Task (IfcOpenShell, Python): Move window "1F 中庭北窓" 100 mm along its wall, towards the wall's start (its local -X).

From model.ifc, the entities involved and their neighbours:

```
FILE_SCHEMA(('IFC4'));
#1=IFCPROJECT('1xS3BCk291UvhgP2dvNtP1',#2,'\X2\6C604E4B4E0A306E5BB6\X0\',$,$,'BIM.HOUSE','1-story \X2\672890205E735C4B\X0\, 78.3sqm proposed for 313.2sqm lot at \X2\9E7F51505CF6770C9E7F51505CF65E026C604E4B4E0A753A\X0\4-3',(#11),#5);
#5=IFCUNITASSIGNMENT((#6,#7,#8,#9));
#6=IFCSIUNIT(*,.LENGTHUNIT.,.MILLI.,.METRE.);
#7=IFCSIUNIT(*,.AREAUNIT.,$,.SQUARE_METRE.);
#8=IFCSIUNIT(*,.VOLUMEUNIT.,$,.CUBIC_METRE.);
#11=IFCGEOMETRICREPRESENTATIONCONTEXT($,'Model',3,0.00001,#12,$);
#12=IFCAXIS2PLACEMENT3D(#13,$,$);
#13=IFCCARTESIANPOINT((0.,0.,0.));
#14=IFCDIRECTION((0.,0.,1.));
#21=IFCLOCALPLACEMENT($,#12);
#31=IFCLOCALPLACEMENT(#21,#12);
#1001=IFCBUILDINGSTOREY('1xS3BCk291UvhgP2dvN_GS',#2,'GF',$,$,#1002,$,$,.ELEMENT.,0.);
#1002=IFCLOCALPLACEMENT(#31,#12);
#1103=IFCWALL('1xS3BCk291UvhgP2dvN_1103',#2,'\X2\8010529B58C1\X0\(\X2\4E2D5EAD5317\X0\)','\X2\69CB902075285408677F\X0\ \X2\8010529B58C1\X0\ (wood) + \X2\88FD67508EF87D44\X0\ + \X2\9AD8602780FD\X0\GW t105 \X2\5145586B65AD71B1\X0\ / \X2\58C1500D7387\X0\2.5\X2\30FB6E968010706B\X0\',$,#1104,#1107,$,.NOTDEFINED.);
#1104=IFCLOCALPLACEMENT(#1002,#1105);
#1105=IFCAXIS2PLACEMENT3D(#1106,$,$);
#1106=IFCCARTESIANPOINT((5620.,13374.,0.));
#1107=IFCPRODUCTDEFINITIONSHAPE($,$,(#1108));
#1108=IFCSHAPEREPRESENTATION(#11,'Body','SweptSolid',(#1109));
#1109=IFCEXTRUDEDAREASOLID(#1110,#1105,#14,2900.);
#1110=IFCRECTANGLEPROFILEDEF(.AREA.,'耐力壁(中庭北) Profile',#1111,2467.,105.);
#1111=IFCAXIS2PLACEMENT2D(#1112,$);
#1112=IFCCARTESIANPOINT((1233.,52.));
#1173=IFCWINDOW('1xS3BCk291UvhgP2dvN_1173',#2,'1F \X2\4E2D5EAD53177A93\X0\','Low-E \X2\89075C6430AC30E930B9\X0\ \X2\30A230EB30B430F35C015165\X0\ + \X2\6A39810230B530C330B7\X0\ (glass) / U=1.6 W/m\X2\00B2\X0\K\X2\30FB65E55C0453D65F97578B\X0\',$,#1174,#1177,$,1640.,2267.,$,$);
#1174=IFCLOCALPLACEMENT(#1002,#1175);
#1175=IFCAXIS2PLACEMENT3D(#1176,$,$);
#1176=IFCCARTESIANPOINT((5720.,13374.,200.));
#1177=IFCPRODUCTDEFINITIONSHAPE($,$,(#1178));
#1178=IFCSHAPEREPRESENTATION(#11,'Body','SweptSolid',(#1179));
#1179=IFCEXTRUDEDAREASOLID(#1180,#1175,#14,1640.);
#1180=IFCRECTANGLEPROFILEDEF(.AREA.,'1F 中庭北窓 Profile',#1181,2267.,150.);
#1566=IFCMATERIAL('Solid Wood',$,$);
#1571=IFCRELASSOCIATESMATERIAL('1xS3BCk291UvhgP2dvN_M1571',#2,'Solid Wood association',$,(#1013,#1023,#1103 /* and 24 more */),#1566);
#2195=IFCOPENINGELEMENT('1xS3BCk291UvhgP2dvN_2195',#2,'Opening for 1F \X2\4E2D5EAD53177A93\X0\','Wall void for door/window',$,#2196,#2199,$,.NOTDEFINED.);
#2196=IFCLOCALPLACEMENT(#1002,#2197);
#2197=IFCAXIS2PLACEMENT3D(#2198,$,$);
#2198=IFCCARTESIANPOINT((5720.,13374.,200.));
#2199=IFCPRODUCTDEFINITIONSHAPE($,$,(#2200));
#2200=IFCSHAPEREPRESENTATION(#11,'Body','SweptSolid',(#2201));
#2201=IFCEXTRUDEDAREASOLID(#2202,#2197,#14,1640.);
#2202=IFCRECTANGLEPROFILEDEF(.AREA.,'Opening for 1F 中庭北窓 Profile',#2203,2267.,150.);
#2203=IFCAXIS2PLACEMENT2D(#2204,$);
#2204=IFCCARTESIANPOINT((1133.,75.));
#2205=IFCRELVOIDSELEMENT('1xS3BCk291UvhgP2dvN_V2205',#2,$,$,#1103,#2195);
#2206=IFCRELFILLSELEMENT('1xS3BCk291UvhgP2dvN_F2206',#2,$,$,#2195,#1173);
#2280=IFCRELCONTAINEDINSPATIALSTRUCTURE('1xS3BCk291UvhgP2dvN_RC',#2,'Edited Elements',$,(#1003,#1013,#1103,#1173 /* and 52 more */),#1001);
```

```python
import ifcopenshell
import ifcopenshell.api.geometry
import ifcopenshell.util.placement

model = ifcopenshell.open("model.ifc")

window = model.by_guid("1xS3BCk291UvhgP2dvN_1173")
opening = window.FillsVoids[0].RelatingOpeningElement
wall = opening.VoidsElements[0].RelatingBuildingElement

wall_matrix = ifcopenshell.util.placement.get_local_placement(wall.ObjectPlacement)
shift = wall_matrix[:3, 0] * -100.0
before = ifcopenshell.util.placement.get_local_placement(window.ObjectPlacement)[:3, 3].copy()

# The window is not placed relative to its opening, so move both.
for product in (opening, window):
    matrix = ifcopenshell.util.placement.get_local_placement(product.ObjectPlacement)
    matrix[:3, 3] += shift
    ifcopenshell.api.geometry.edit_object_placement(model, product=product, matrix=matrix, is_si=False)

after = ifcopenshell.util.placement.get_local_placement(window.ObjectPlacement)[:3, 3]
print("window moved by", (after - before).round(3) + 0.0)

model.write("model_edited.ifc")
```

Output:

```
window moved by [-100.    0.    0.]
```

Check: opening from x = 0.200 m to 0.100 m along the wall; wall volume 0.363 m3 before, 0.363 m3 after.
